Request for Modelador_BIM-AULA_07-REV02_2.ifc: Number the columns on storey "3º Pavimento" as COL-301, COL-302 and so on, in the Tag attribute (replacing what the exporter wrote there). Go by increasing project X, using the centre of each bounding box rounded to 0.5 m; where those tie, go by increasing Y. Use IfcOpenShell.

First a look at what the model holds.

```python
import ifcopenshell
import ifcopenshell.util.element
import ifcopenshell.util.placement

model = ifcopenshell.open("Modelador_BIM-AULA_07-REV02_2.ifc")
print(model.schema)
storey = next(s for s in model.by_type("IfcBuildingStorey") if s.Name == "3º Pavimento")
columns = [e for e in ifcopenshell.util.element.get_decomposition(storey) if e.is_a("IfcColumn")]
for e in sorted(columns, key=lambda e: e.id()):
    origin = ifcopenshell.util.placement.get_local_placement(e.ObjectPlacement)[:3, 3]
    print(e.id(), e.Tag, e.Name, origin.round(2) + 0.0, sep=" | ")
```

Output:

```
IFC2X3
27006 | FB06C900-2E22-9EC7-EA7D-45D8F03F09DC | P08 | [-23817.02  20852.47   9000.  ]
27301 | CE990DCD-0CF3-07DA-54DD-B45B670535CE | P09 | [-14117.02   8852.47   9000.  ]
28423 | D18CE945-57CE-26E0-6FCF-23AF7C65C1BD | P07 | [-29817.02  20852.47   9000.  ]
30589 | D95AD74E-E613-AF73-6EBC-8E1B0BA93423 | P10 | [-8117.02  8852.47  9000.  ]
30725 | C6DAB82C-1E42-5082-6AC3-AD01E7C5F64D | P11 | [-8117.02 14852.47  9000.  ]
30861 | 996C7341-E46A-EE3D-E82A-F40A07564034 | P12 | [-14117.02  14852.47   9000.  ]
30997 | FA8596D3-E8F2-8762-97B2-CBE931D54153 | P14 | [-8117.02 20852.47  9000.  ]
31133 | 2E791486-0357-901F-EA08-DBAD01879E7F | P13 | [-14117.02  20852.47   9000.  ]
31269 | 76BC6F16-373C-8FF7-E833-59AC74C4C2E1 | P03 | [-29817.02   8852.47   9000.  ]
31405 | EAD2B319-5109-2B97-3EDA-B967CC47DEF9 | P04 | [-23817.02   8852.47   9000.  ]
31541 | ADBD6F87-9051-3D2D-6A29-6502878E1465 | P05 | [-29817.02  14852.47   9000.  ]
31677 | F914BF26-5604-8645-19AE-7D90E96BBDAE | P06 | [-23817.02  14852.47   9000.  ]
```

```python
import ifcopenshell
import ifcopenshell.geom
import ifcopenshell.util.element
import ifcopenshell.util.shape

model = ifcopenshell.open("Modelador_BIM-AULA_07-REV02_2.ifc")
settings = ifcopenshell.geom.settings()
settings.set("use-world-coords", True)


def centre(element):
    shape = ifcopenshell.geom.create_shape(settings, element)
    return ifcopenshell.util.shape.get_bbox_centroid(shape.geometry)


storey = next(s for s in model.by_type("IfcBuildingStorey") if s.Name == "3º Pavimento")
columns = [e for e in ifcopenshell.util.element.get_decomposition(storey) if e.is_a("IfcColumn")]

# Insertion points can sit at a corner or the storey origin, so sort by the geometry (in metres).
centres = {e: centre(e) for e in columns}
columns.sort(key=lambda e: (round(centres[e][0] / 0.5), centres[e][1]))

for i, e in enumerate(columns, start=1):
    number = f"COL-3{i:02d}"
    e.Tag = number
    print(e.id(), number)

model.write("Modelador_BIM-AULA_07-REV02_2_edited.ifc")
```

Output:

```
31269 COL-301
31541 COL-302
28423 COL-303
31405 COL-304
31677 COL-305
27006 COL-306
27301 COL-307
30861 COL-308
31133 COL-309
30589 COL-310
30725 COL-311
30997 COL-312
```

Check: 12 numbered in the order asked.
